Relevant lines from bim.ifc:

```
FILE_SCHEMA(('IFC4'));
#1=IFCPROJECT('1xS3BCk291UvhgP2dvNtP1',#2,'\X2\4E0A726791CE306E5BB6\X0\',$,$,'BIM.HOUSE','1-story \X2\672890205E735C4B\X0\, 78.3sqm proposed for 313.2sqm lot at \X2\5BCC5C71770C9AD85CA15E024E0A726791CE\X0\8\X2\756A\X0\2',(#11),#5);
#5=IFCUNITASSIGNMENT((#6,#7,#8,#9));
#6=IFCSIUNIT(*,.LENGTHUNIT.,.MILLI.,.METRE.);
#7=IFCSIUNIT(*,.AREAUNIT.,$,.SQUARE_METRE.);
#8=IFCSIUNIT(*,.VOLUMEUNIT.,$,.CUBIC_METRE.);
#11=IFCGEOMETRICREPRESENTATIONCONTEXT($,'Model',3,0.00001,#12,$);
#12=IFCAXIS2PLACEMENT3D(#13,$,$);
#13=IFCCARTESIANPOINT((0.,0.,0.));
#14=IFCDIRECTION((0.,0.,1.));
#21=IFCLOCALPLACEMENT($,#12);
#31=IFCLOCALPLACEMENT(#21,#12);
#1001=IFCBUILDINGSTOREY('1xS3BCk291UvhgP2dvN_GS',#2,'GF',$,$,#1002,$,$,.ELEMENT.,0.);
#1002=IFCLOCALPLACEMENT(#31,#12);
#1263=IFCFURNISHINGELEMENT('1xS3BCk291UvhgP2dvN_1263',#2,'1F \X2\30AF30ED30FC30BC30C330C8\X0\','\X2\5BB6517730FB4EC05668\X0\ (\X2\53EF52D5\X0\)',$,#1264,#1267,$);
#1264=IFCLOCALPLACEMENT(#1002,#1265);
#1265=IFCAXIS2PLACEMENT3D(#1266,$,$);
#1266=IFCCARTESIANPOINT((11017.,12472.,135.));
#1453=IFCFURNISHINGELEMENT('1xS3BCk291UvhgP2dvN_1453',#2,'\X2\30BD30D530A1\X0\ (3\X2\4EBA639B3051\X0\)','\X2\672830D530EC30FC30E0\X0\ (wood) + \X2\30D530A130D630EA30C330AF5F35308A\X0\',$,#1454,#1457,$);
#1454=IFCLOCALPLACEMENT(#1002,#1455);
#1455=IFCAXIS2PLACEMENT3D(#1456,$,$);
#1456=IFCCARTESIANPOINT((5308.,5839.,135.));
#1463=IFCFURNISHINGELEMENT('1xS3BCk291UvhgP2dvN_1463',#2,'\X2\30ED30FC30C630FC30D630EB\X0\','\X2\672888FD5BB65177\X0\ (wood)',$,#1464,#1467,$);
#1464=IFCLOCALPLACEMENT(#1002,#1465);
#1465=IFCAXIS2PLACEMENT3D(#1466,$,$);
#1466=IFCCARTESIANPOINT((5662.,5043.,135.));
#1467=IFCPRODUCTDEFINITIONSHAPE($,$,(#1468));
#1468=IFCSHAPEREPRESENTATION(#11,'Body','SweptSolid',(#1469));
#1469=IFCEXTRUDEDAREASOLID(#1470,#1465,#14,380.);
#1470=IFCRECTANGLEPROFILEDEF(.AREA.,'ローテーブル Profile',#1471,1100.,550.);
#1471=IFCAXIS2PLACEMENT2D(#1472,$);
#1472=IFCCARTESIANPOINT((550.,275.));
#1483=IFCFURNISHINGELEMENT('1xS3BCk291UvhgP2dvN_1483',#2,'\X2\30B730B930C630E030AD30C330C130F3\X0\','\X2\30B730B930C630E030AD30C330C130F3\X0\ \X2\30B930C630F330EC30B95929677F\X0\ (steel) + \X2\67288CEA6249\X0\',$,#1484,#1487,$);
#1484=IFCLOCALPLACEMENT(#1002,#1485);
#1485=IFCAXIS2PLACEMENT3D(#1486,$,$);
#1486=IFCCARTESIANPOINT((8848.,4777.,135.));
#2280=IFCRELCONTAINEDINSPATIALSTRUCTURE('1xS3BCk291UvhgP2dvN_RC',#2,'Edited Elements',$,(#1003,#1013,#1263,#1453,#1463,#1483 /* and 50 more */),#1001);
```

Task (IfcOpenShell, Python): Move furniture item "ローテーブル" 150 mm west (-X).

```python
import ifcopenshell
import ifcopenshell.api.geometry
import ifcopenshell.util.placement
import ifcopenshell.util.unit

model = ifcopenshell.open("bim.ifc")
unit_scale = ifcopenshell.util.unit.calculate_unit_scale(model)

item = model.by_guid("1xS3BCk291UvhgP2dvN_1463")
matrix = ifcopenshell.util.placement.get_local_placement(item.ObjectPlacement)
matrix[0, 3] -= 0.15 / unit_scale
ifcopenshell.api.geometry.edit_object_placement(model, product=item, matrix=matrix, is_si=False)

print(ifcopenshell.util.placement.get_local_placement(item.ObjectPlacement).round(3) + 0.0)

model.write("bim_v2.ifc")
```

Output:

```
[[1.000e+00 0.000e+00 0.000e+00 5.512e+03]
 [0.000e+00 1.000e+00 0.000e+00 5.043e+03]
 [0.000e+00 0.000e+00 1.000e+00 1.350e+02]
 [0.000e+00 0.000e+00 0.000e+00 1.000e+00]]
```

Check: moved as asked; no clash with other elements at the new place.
